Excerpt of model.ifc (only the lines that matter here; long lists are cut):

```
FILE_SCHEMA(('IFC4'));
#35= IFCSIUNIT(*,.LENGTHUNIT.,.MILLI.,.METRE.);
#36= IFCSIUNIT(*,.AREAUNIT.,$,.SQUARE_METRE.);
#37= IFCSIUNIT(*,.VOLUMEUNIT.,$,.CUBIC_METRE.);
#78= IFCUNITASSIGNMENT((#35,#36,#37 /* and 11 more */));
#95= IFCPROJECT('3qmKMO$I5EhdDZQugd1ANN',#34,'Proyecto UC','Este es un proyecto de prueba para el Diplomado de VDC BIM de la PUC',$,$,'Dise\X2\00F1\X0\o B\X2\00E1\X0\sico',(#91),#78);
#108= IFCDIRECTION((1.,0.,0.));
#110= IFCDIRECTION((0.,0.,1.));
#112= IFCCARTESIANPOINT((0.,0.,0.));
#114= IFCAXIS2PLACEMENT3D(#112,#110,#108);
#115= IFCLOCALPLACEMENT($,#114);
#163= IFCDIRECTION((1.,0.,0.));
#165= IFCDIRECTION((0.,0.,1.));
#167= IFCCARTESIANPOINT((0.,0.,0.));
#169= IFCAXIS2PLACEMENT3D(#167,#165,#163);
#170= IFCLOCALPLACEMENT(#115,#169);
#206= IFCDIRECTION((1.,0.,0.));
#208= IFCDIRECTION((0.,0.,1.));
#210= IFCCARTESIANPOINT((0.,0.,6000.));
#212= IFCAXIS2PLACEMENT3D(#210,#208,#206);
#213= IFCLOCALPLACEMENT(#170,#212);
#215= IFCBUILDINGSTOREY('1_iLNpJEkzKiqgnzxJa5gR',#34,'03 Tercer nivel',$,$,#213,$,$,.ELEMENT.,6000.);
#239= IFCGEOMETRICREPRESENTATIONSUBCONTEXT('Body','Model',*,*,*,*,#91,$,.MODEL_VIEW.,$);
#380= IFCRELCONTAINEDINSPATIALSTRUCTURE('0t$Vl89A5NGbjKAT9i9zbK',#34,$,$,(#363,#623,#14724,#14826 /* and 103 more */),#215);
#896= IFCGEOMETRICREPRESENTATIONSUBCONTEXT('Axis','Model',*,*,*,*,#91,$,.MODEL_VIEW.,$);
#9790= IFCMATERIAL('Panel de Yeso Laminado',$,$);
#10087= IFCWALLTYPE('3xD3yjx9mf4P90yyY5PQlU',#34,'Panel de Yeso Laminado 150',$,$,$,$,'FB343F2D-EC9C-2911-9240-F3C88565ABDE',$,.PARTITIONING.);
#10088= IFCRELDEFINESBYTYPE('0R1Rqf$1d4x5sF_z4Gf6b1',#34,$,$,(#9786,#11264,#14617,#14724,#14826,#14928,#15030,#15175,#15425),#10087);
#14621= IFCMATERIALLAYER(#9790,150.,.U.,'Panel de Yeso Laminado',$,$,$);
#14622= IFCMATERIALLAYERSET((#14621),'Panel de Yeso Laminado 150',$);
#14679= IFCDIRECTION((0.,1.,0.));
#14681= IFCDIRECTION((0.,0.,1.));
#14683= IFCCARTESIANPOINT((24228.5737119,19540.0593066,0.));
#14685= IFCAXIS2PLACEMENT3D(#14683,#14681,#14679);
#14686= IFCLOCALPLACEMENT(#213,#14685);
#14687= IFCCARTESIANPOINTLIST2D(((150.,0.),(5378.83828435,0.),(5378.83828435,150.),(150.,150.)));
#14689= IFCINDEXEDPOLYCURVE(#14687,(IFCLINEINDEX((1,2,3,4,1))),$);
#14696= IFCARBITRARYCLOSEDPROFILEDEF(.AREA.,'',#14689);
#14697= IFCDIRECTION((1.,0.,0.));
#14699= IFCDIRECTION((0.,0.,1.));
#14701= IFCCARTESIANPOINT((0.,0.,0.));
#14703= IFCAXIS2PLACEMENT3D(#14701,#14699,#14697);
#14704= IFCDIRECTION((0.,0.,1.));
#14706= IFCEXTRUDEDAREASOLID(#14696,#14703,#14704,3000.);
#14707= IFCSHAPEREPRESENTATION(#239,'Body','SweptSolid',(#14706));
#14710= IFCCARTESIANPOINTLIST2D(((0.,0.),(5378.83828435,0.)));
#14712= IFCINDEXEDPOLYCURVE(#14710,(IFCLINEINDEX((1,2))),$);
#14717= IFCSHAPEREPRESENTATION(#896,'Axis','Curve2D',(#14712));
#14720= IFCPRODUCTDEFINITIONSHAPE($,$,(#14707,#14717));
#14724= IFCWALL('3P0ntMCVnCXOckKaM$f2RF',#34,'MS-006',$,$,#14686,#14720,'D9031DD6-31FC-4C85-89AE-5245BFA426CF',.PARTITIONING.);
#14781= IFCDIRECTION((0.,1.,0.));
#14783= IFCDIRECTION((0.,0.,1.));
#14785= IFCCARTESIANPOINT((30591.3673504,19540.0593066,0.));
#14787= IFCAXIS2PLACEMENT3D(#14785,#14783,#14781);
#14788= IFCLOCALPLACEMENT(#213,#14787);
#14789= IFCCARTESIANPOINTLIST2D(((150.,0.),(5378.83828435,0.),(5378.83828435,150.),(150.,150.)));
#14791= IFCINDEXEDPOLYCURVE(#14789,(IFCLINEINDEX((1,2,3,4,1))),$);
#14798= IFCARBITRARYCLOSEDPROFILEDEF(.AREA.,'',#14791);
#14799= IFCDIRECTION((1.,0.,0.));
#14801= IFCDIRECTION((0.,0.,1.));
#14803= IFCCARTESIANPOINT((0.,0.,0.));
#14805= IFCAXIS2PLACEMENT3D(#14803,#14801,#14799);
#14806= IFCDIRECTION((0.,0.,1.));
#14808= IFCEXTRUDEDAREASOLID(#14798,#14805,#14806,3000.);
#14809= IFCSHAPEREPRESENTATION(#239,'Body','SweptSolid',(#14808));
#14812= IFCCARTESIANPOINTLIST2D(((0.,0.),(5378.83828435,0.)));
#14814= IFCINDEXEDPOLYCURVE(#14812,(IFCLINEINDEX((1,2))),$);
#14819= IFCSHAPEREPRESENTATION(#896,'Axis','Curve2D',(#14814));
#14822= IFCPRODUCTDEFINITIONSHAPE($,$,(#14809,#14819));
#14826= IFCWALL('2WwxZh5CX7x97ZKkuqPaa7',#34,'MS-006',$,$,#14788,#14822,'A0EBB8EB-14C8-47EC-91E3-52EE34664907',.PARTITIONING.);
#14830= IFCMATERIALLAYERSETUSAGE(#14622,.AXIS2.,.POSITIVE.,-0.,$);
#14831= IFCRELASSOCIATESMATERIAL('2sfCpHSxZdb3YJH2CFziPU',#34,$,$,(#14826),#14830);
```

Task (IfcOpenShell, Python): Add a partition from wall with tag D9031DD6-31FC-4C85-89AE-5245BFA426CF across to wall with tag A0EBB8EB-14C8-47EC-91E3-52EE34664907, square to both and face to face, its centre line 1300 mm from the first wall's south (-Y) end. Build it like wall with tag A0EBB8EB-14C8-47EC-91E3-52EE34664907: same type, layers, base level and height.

```python
import numpy as np
import ifcopenshell
import ifcopenshell.api.geometry
import ifcopenshell.api.material
import ifcopenshell.api.pset
import ifcopenshell.api.root
import ifcopenshell.api.spatial
import ifcopenshell.api.type
import ifcopenshell.geom
import ifcopenshell.util.element
import ifcopenshell.util.placement
import ifcopenshell.util.representation
import ifcopenshell.util.shape
import ifcopenshell.util.unit

model = ifcopenshell.open("model.ifc")
unit_scale = ifcopenshell.util.unit.calculate_unit_scale(model)
settings = ifcopenshell.geom.settings()
settings.set("use-world-coords", True)

start_wall = model.by_guid("3P0ntMCVnCXOckKaM$f2RF")
end_wall = model.by_id(14826)
like = model.by_id(14826)
matrix = ifcopenshell.util.placement.get_local_placement(start_wall.ObjectPlacement)
matrix[:3, 3] *= unit_scale


def extent(element):
    """Bounding box in the first wall's axes, in metres."""
    shape = ifcopenshell.geom.create_shape(settings, element)
    points = (ifcopenshell.util.shape.get_vertices(shape.geometry) - matrix[:3, 3]) @ matrix[:3, :3]
    return points.min(axis=0), points.max(axis=0)


y_start = extent(start_wall)[0][1]
y_end = extent(end_wall)[1][1]
like_min, like_max = extent(like)
length, height = float(abs(y_end - y_start)), float(like_max[2] - like_min[2])
layer_set = ifcopenshell.util.element.get_material(like, should_skip_usage=True)
thickness = sum(layer.LayerThickness for layer in layer_set.MaterialLayers) * unit_scale

wall = ifcopenshell.api.root.create_entity(model, ifc_class="IfcWall", name="New partition")
storey = ifcopenshell.util.element.get_container(like)
ifcopenshell.api.spatial.assign_container(model, products=[wall], relating_structure=storey)
ifcopenshell.api.type.assign_type(
    model, related_objects=[wall], relating_type=ifcopenshell.util.element.get_type(like), should_map_representations=False
)
rel = ifcopenshell.api.material.assign_material(
    model, products=[wall], type="IfcMaterialLayerSetUsage", material=layer_set
)
rel.RelatingMaterial.OffsetFromReferenceLine = -thickness / 2 / unit_scale
pset = ifcopenshell.api.pset.add_pset(model, product=wall, name="Pset_WallCommon")
ifcopenshell.api.pset.edit_pset(model, pset=pset, properties={"IsExternal": False, "LoadBearing": False})

# The axis runs down the middle of the wall.
axis = ifcopenshell.api.geometry.add_axis_representation(
    model, context=ifcopenshell.util.representation.get_context(model, "Model", "Axis"), axis=[(0.0, 0.0), (length, 0.0)]
)
body = ifcopenshell.api.geometry.add_wall_representation(
    model,
    context=ifcopenshell.util.representation.get_context(model, "Model", "Body", "MODEL_VIEW"),
    length=length,
    height=height,
    thickness=thickness,
    offset=-thickness / 2,
)
for representation in (axis, body):
    ifcopenshell.api.geometry.assign_representation(model, product=wall, representation=representation)

placement = matrix @ ifcopenshell.util.placement.rotation(-90, "Z")
placement[:, 3] = matrix @ np.array([extent(start_wall)[0][0] + 1.3, y_start, like_min[2], 1.0])
ifcopenshell.api.geometry.edit_object_placement(model, product=wall, matrix=placement)

print(f"partition {length:.3f} m long, {height:.3f} m high, {thickness:.3f} m thick")

model.write("model_edited.ifc")
```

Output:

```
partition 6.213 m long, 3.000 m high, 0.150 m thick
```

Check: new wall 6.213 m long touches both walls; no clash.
